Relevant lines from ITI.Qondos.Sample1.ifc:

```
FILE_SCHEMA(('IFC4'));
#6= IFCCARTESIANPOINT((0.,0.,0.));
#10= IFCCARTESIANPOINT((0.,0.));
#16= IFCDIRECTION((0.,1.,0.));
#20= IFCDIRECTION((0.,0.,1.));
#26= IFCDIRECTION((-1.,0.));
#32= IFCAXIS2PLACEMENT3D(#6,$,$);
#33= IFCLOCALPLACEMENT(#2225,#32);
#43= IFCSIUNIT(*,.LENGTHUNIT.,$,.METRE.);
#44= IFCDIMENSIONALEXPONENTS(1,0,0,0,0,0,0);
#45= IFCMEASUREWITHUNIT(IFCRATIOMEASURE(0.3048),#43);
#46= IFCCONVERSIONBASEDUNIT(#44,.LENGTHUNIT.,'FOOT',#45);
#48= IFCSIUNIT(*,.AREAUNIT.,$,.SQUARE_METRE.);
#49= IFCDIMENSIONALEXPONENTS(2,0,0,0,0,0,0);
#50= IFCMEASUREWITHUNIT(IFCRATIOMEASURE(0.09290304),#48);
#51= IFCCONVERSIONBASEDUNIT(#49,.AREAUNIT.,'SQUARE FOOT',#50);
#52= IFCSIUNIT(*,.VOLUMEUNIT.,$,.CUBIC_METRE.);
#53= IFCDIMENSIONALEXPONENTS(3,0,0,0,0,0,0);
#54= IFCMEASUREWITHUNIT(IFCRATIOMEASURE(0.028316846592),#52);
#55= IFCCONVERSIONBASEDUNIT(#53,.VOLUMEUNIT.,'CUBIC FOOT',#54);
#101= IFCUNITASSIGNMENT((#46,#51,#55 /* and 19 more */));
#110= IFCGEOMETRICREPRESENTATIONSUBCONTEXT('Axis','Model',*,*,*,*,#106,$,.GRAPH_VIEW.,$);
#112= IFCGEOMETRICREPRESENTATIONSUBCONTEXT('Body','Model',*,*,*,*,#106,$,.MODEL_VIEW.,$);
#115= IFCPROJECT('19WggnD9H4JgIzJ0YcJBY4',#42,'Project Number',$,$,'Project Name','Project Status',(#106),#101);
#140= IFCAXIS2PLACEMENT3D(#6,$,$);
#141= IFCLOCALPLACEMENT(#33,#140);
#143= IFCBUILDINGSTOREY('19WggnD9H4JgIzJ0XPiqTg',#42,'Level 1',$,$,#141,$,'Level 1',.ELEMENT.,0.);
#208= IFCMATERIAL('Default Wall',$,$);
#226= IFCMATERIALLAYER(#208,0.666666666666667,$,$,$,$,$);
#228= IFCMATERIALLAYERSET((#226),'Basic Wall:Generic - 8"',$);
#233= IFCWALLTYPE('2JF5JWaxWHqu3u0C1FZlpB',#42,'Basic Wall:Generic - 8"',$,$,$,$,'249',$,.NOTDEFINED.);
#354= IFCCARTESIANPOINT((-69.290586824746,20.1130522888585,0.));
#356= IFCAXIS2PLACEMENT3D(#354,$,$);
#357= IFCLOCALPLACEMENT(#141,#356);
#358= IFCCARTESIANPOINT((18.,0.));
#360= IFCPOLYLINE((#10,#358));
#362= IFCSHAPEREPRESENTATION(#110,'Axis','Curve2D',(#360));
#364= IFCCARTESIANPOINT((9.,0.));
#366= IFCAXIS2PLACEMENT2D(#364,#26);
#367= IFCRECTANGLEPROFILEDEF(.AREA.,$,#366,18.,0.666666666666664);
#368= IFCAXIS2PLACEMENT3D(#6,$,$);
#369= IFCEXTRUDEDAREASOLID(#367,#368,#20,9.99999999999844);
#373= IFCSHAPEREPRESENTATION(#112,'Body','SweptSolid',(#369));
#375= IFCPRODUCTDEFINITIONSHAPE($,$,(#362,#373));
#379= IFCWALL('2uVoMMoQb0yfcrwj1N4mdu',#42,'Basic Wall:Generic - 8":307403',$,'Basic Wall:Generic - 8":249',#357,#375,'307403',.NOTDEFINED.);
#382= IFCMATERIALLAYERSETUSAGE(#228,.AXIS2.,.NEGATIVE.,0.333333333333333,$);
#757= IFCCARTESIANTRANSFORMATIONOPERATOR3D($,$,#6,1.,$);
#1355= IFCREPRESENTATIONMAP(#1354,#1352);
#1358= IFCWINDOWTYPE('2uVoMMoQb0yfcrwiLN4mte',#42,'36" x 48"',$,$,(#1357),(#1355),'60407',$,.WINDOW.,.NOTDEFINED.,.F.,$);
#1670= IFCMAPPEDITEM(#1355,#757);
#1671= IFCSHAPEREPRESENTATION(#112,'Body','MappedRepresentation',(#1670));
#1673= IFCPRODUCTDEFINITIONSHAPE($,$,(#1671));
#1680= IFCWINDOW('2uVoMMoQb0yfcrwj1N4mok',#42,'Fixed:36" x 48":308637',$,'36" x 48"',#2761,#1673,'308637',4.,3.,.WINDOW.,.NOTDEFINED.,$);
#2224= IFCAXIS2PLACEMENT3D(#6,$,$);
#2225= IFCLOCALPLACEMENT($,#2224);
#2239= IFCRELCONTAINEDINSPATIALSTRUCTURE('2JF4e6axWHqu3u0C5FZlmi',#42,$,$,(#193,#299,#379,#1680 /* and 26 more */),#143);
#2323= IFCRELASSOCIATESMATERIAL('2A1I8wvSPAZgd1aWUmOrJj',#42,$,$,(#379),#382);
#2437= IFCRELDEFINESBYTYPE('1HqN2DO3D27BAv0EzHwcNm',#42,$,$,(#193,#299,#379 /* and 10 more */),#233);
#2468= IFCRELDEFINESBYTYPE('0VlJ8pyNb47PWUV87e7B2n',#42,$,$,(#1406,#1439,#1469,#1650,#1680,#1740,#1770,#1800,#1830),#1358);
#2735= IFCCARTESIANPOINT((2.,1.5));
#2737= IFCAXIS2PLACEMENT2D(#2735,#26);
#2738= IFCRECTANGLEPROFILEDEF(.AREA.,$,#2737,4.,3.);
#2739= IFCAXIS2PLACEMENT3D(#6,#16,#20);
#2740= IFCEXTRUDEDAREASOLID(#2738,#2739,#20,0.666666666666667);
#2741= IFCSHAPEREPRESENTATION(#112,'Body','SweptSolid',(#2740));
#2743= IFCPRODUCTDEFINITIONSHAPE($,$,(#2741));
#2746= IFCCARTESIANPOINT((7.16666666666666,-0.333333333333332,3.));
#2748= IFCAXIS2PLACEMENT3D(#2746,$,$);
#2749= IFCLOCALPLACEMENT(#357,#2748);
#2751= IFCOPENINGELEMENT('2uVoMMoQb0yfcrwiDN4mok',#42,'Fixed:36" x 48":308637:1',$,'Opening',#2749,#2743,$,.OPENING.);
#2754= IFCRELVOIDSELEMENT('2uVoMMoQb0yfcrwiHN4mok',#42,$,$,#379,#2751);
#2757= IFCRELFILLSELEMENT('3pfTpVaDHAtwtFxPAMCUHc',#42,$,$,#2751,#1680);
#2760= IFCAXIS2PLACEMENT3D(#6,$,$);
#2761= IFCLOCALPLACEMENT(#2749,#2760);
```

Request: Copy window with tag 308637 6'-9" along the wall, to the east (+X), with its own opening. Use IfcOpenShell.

```python
import ifcopenshell
import ifcopenshell.api.feature
import ifcopenshell.api.geometry
import ifcopenshell.api.root
import ifcopenshell.geom
import ifcopenshell.util.element
import ifcopenshell.util.placement
import ifcopenshell.util.shape
import ifcopenshell.util.unit

model = ifcopenshell.open("ITI.Qondos.Sample1.ifc")
unit_scale = ifcopenshell.util.unit.calculate_unit_scale(model)
settings = ifcopenshell.geom.settings()


def volume(element):
    """Net volume in cubic metres, openings subtracted."""
    shape = ifcopenshell.geom.create_shape(settings, element)
    return ifcopenshell.util.shape.get_volume(shape.geometry)


def reuse_history(source, copy):
    """copy_class also copies each property set's owner history, people and application; keep the originals."""
    for rel in copy.IsDefinedBy:
        if rel.is_a("IfcRelDefinesByProperties") and (history := rel.RelatingPropertyDefinition.OwnerHistory):
            rel.RelatingPropertyDefinition.OwnerHistory = source.OwnerHistory
            ifcopenshell.util.element.remove_deep2(model, history)


window = model.by_guid("2uVoMMoQb0yfcrwj1N4mok")
opening = window.FillsVoids[0].RelatingOpeningElement
wall = opening.VoidsElements[0].RelatingBuildingElement
before = volume(wall)
shift = ifcopenshell.util.placement.get_local_placement(wall.ObjectPlacement)[:3, 0] * 81 * 0.0254 / unit_scale

# copy_class copies the void relationship, type, container and properties, but no geometry.
new_opening = ifcopenshell.api.root.copy_class(model, product=opening)
new_opening.Representation = ifcopenshell.util.element.copy_deep(
    model, opening.Representation, exclude=["IfcGeometricRepresentationContext", "IfcRepresentationMap"]
)
new_opening.Name = 'Fixed:36" x 48"'
new_window = ifcopenshell.api.root.copy_class(model, product=window)
new_window.Representation = ifcopenshell.util.element.copy_deep(
    model, window.Representation, exclude=["IfcGeometricRepresentationContext", "IfcRepresentationMap"]
)
new_window.Name = 'Fixed:36" x 48"'
new_window.Tag = None
reuse_history(window, new_window)
ifcopenshell.api.feature.add_filling(model, opening=new_opening, element=new_window)

for old, new in ((opening, new_opening), (window, new_window)):
    matrix = ifcopenshell.util.placement.get_local_placement(old.ObjectPlacement)
    matrix[:3, 3] += shift
    ifcopenshell.api.geometry.edit_object_placement(model, product=new, matrix=matrix, is_si=False)

after = volume(wall)

print(f"wall volume {before:.3f} -> {after:.3f} m3")

model.write("ITI.Qondos.Sample1_updated.ifc")
```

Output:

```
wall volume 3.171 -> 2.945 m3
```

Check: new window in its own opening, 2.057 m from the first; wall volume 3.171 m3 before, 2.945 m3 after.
